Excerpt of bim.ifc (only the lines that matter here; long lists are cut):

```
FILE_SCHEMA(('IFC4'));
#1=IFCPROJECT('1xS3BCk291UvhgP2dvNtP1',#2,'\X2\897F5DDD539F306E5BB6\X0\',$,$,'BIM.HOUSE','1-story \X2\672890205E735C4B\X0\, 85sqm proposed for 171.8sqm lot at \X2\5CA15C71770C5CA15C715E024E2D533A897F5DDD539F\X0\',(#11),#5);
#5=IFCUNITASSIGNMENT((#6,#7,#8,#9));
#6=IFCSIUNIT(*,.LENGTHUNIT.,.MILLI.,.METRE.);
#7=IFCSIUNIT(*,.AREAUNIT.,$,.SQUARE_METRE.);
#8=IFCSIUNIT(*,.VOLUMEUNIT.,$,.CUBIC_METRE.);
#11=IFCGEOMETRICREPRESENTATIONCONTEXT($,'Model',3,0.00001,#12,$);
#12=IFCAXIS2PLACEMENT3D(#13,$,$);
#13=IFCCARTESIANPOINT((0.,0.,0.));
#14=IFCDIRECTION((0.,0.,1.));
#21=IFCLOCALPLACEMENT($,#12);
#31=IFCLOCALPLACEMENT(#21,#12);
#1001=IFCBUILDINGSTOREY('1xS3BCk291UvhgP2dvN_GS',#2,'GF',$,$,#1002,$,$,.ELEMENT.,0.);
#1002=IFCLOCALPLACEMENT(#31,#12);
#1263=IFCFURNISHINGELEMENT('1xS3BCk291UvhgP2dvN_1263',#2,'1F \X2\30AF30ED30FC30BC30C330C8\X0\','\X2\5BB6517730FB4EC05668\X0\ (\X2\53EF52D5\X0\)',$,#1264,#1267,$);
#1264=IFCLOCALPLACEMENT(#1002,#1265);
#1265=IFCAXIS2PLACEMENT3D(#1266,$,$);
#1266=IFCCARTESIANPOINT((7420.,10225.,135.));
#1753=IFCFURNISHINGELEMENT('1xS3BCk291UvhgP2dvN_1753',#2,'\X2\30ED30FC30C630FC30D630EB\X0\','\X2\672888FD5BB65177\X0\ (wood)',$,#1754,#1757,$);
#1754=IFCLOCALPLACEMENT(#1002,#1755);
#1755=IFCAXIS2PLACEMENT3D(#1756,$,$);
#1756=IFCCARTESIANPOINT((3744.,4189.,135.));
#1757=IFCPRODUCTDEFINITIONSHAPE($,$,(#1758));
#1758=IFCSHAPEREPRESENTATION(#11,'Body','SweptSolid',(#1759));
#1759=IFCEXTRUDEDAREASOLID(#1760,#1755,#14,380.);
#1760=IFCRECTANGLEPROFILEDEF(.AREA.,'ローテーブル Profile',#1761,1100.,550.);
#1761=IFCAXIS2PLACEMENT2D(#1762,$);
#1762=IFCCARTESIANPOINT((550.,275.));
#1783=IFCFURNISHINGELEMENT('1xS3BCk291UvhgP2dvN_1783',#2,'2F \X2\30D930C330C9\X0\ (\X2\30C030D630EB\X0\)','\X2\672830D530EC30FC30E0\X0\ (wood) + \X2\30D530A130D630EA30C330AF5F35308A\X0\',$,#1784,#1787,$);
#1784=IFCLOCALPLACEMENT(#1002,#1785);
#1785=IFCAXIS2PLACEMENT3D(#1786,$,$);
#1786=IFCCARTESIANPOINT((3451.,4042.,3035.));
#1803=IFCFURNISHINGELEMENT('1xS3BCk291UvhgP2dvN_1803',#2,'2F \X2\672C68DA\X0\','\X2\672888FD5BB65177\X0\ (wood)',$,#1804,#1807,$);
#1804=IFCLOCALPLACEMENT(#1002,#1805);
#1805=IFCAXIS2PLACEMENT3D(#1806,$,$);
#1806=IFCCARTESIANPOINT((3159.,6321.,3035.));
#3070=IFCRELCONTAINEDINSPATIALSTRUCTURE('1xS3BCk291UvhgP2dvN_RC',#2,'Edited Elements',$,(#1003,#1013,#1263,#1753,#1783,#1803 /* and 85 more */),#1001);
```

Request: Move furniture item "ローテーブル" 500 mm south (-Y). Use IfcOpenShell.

```python
import ifcopenshell
import ifcopenshell.api.geometry
import ifcopenshell.util.placement
import ifcopenshell.util.unit

model = ifcopenshell.open("bim.ifc")
unit_scale = ifcopenshell.util.unit.calculate_unit_scale(model)

item = model.by_id(1753)
matrix = ifcopenshell.util.placement.get_local_placement(item.ObjectPlacement)
matrix[1, 3] -= 0.5 / unit_scale
ifcopenshell.api.geometry.edit_object_placement(model, product=item, matrix=matrix, is_si=False)

print(ifcopenshell.util.placement.get_local_placement(item.ObjectPlacement).round(3) + 0.0)

model.write("bim-out.ifc")
```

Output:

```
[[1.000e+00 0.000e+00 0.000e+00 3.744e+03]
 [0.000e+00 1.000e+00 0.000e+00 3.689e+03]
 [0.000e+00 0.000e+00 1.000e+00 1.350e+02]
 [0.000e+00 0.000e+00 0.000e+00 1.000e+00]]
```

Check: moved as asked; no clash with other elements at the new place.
